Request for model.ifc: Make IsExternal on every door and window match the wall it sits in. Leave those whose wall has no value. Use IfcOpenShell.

First a look at what the model holds.

```python
import ifcopenshell
import ifcopenshell.util.element

model = ifcopenshell.open("model.ifc")
print(model.schema)
seen = {}
for e in model.by_type("IfcDoor") + model.by_type("IfcWindow"):
    if not e.FillsVoids:
        continue
    host = e.FillsVoids[0].RelatingOpeningElement.VoidsElements[0].RelatingBuildingElement
    own = ifcopenshell.util.element.get_pset(e, f"Pset_{e.is_a()[3:].removesuffix('StandardCase')}Common", "IsExternal")
    wall = ifcopenshell.util.element.get_pset(host, "Pset_WallCommon", "IsExternal")
    seen[e.is_a(), own, wall] = seen.get((e.is_a(), own, wall), 0) + 1
for (cls, own, wall), count in sorted(seen.items(), key=str):
    print(count, cls, "IsExternal:", own, "| host wall:", wall)
```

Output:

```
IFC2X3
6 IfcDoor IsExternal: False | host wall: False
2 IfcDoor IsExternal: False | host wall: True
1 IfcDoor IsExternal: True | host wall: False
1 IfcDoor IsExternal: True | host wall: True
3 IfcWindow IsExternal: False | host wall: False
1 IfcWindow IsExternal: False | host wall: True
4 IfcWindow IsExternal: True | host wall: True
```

```python
import ifcopenshell
import ifcopenshell.api.pset
import ifcopenshell.util.element

model = ifcopenshell.open("model.ifc")

count = 0
for ifc_class, pset_name in (("IfcDoor", "Pset_DoorCommon"), ("IfcWindow", "Pset_WindowCommon")):
    for e in model.by_type(ifc_class):
        if not e.FillsVoids:
            continue
        host = e.FillsVoids[0].RelatingOpeningElement.VoidsElements[0].RelatingBuildingElement
        external = ifcopenshell.util.element.get_pset(host, "Pset_WallCommon", "IsExternal")
        if external is None or ifcopenshell.util.element.get_pset(e, pset_name, "IsExternal") == external:
            continue
        pset = ifcopenshell.api.pset.add_pset(model, product=e, name=pset_name)
        ifcopenshell.api.pset.edit_pset(model, pset=pset, properties={"IsExternal": external})
        count += 1

print(count, "updated")

model.write("model_edited.ifc")
```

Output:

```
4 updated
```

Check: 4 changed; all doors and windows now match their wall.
